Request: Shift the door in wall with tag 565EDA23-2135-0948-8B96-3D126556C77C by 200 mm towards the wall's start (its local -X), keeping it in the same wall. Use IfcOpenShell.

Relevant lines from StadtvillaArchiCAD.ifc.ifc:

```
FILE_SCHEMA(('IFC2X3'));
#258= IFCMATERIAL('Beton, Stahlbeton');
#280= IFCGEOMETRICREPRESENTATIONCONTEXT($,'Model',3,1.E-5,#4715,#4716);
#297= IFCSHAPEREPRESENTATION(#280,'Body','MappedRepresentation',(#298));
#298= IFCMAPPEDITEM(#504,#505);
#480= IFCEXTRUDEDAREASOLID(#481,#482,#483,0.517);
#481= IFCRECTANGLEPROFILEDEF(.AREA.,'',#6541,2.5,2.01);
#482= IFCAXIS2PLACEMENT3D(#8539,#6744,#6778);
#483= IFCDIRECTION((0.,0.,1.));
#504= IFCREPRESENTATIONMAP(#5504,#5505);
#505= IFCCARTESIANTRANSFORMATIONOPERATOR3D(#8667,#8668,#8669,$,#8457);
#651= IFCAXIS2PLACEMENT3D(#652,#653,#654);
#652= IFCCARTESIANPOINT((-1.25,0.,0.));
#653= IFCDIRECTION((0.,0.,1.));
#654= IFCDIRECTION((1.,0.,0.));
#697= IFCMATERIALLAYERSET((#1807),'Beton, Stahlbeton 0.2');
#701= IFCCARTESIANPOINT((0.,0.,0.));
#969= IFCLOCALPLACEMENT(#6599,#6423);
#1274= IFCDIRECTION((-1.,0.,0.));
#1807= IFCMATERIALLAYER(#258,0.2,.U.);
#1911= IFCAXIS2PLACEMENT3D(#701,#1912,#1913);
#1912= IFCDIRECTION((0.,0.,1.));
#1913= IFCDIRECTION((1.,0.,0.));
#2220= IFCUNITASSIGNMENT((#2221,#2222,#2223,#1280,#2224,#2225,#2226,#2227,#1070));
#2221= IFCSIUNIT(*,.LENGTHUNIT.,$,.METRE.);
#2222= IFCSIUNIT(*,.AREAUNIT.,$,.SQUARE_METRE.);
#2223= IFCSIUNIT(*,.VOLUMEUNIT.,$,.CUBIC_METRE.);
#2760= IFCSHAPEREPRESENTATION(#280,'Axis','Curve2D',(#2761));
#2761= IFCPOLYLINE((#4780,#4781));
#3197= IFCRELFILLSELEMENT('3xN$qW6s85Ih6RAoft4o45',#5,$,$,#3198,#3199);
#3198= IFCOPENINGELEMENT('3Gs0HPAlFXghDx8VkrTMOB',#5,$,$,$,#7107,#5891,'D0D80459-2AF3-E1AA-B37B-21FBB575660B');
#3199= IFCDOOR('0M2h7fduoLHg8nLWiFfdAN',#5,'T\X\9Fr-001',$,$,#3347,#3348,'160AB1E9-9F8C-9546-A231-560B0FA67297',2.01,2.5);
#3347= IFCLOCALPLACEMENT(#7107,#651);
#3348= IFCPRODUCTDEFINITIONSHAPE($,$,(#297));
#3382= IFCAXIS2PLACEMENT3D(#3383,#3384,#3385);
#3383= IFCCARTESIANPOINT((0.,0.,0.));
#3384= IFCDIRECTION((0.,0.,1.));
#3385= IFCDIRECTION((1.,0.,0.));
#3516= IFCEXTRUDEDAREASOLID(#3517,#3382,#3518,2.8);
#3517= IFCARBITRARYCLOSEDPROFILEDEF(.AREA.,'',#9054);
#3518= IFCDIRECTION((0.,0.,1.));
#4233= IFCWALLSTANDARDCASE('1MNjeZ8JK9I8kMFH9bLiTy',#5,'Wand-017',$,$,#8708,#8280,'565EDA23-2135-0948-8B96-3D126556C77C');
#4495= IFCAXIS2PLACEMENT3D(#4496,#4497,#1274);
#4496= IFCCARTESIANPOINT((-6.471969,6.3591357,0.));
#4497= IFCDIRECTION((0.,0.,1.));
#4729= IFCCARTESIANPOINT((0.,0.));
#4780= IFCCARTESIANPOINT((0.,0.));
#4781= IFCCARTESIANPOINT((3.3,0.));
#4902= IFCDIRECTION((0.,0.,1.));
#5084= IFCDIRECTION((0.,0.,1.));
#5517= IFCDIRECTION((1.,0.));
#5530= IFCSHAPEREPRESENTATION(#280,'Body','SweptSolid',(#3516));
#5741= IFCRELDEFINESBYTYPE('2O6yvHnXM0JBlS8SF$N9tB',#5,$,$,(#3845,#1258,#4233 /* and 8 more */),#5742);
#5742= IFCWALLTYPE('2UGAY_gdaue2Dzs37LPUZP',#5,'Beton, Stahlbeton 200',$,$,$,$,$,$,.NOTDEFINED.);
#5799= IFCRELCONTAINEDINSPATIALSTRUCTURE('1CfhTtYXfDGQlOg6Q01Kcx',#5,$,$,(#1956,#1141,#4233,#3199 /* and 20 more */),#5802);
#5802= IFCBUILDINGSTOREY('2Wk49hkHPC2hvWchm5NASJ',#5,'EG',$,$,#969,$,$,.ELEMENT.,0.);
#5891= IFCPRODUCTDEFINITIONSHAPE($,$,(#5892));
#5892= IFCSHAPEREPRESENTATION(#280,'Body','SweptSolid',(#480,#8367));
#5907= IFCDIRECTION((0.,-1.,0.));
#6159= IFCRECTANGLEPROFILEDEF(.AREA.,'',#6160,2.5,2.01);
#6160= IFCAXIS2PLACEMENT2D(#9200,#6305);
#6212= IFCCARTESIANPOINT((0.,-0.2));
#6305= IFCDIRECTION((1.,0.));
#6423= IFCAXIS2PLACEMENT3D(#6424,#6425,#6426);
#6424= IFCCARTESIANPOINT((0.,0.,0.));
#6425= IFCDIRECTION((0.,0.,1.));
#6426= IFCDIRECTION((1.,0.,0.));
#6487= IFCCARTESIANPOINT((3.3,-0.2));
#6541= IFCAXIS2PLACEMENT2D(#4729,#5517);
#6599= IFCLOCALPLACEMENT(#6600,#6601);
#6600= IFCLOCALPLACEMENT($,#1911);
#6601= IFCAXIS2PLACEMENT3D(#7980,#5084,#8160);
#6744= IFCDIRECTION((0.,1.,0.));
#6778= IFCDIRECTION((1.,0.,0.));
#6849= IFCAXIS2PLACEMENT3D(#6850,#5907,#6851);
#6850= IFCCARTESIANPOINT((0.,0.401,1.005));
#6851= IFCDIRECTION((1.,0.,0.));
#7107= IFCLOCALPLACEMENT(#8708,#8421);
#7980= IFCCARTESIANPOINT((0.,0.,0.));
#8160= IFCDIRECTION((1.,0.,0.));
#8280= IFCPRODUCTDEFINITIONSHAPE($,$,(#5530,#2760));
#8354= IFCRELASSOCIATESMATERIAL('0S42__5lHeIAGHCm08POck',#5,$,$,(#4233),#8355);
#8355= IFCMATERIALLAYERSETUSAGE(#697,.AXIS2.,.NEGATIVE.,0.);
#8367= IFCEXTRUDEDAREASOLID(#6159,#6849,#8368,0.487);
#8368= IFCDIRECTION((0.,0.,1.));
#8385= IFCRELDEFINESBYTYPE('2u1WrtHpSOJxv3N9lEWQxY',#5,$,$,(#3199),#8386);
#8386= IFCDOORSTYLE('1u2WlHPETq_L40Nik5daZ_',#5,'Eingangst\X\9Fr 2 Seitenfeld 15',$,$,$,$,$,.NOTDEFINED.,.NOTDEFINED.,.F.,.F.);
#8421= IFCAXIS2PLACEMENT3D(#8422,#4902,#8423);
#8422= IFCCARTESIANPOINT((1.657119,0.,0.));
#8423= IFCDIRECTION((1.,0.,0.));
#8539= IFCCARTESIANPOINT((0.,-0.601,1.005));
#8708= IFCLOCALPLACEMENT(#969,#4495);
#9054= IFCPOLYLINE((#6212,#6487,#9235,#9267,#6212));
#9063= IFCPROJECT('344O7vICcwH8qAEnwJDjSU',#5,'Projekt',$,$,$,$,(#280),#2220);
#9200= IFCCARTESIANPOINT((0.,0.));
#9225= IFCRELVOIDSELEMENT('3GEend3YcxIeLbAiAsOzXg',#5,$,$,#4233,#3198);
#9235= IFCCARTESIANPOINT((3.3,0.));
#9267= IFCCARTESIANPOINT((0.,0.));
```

```python
import ifcopenshell
import ifcopenshell.api.geometry
import ifcopenshell.util.placement

model = ifcopenshell.open("StadtvillaArchiCAD.ifc.ifc")

door = model.by_id(3199)
opening = door.FillsVoids[0].RelatingOpeningElement
wall = opening.VoidsElements[0].RelatingBuildingElement

wall_matrix = ifcopenshell.util.placement.get_local_placement(wall.ObjectPlacement)
shift = wall_matrix[:3, 0] * -0.2
before = ifcopenshell.util.placement.get_local_placement(door.ObjectPlacement)[:3, 3].copy()

# The door is placed relative to its opening, so it follows when the opening moves.
matrix = ifcopenshell.util.placement.get_local_placement(opening.ObjectPlacement)
matrix[:3, 3] += shift
ifcopenshell.api.geometry.edit_object_placement(
    model, product=opening, matrix=matrix, is_si=False, should_transform_children=True
)

after = ifcopenshell.util.placement.get_local_placement(door.ObjectPlacement)[:3, 3]
print("door moved by", (after - before).round(3) + 0.0)

model.write("StadtvillaArchiCAD.ifc_rev.ifc")
```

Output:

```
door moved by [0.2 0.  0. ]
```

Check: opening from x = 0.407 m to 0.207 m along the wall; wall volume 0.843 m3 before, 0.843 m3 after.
